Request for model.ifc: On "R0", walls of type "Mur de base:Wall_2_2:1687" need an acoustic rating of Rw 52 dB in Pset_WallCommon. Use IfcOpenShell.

First a look at what the model holds.

```python
import ifcopenshell
import ifcopenshell.util.element

model = ifcopenshell.open("model.ifc")
print(model.schema)
storey = next(s for s in model.by_type("IfcBuildingStorey") if s.Name == "R0")
walls = [e for e in ifcopenshell.util.element.get_decomposition(storey) if e.is_a("IfcWall")]
seen = {}
for e in walls:
    element_type = ifcopenshell.util.element.get_type(e)
    key = (element_type.Name if element_type != e and element_type else None, ifcopenshell.util.element.get_pset(e, "Pset_WallCommon", "AcousticRating"))
    seen[key] = seen.get(key, 0) + 1
for (name, value), count in sorted(seen.items(), key=str):
    print(count, "x", name, "|", value)
```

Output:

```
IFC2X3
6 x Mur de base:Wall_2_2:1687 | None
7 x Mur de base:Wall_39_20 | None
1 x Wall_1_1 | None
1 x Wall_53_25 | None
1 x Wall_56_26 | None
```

```python
import ifcopenshell
import ifcopenshell.api.pset
import ifcopenshell.util.element

model = ifcopenshell.open("model.ifc")

storey = next(s for s in model.by_type("IfcBuildingStorey") if s.Name == "R0")
walls = [e for e in ifcopenshell.util.element.get_decomposition(storey) if e.is_a("IfcWall")]

count = 0
for e in walls:
    element_type = ifcopenshell.util.element.get_type(e)
    if element_type in (None, e) or element_type.Name != "Mur de base:Wall_2_2:1687":
        continue
    # add_pset returns the element's existing set when there is one.
    pset = ifcopenshell.api.pset.add_pset(model, product=e, name="Pset_WallCommon")
    ifcopenshell.api.pset.edit_pset(model, pset=pset, properties={"AcousticRating": "Rw 52 dB"})
    count += 1

print(count, "walls updated")

model.write("model-out.ifc")
```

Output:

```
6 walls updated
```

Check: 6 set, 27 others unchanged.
